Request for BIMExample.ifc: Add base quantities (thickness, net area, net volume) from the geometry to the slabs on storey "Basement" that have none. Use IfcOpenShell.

First a look at what the model holds.

```python
import ifcopenshell
import ifcopenshell.util.element
import ifcopenshell.util.unit

model = ifcopenshell.open("BIMExample.ifc")
print(model.schema)
for unit_type in ("LENGTHUNIT", "AREAUNIT", "VOLUMEUNIT"):
    print(unit_type, ifcopenshell.util.unit.calculate_unit_scale(model, unit_type))
storey = next(s for s in model.by_type("IfcBuildingStorey") if s.Name == "Basement")
slabs = [e for e in ifcopenshell.util.element.get_decomposition(storey) if e.is_a("IfcSlab")]
for e in sorted(slabs, key=lambda e: e.id()):
    print(e.id(), e.is_a(), e.Name, list(ifcopenshell.util.element.get_psets(e, qtos_only=True)), sep=" | ")
```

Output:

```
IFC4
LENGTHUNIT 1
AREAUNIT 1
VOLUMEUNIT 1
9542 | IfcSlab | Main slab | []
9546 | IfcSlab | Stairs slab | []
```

```python
import ifcopenshell
import ifcopenshell.api.pset
import ifcopenshell.geom
import ifcopenshell.util.element
import ifcopenshell.util.shape
import ifcopenshell.util.unit

model = ifcopenshell.open("BIMExample.ifc")
unit_scale = ifcopenshell.util.unit.calculate_unit_scale(model)
area_scale = ifcopenshell.util.unit.calculate_unit_scale(model, "AREAUNIT")
volume_scale = ifcopenshell.util.unit.calculate_unit_scale(model, "VOLUMEUNIT")
settings = ifcopenshell.geom.settings()

storey = next(s for s in model.by_type("IfcBuildingStorey") if s.Name == "Basement")
slabs = [e for e in ifcopenshell.util.element.get_decomposition(storey) if e.is_a("IfcSlab")]

for e in sorted(slabs, key=lambda e: e.id()):
    if ifcopenshell.util.element.get_psets(e, qtos_only=True, should_inherit=False):
        continue
    # Geometry comes back in metres, in the element's own axes.
    shape = ifcopenshell.geom.create_shape(settings, e)
    values = {
        "Width": ifcopenshell.util.shape.get_z(shape.geometry) / unit_scale,
        "NetArea": ifcopenshell.util.shape.get_footprint_area(shape.geometry) / area_scale,
        "NetVolume": ifcopenshell.util.shape.get_volume(shape.geometry) / volume_scale,
    }
    qto = ifcopenshell.api.pset.add_qto(model, product=e, name="Qto_SlabBaseQuantities")
    ifcopenshell.api.pset.edit_qto(model, qto=qto, properties=values)
    print(e.id(), {k: round(v, 3) for k, v in values.items()})

model.write("BIMExample-out.ifc")
```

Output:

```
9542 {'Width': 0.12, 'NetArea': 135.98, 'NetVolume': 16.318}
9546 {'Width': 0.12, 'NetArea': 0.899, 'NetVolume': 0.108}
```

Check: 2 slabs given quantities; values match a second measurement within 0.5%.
